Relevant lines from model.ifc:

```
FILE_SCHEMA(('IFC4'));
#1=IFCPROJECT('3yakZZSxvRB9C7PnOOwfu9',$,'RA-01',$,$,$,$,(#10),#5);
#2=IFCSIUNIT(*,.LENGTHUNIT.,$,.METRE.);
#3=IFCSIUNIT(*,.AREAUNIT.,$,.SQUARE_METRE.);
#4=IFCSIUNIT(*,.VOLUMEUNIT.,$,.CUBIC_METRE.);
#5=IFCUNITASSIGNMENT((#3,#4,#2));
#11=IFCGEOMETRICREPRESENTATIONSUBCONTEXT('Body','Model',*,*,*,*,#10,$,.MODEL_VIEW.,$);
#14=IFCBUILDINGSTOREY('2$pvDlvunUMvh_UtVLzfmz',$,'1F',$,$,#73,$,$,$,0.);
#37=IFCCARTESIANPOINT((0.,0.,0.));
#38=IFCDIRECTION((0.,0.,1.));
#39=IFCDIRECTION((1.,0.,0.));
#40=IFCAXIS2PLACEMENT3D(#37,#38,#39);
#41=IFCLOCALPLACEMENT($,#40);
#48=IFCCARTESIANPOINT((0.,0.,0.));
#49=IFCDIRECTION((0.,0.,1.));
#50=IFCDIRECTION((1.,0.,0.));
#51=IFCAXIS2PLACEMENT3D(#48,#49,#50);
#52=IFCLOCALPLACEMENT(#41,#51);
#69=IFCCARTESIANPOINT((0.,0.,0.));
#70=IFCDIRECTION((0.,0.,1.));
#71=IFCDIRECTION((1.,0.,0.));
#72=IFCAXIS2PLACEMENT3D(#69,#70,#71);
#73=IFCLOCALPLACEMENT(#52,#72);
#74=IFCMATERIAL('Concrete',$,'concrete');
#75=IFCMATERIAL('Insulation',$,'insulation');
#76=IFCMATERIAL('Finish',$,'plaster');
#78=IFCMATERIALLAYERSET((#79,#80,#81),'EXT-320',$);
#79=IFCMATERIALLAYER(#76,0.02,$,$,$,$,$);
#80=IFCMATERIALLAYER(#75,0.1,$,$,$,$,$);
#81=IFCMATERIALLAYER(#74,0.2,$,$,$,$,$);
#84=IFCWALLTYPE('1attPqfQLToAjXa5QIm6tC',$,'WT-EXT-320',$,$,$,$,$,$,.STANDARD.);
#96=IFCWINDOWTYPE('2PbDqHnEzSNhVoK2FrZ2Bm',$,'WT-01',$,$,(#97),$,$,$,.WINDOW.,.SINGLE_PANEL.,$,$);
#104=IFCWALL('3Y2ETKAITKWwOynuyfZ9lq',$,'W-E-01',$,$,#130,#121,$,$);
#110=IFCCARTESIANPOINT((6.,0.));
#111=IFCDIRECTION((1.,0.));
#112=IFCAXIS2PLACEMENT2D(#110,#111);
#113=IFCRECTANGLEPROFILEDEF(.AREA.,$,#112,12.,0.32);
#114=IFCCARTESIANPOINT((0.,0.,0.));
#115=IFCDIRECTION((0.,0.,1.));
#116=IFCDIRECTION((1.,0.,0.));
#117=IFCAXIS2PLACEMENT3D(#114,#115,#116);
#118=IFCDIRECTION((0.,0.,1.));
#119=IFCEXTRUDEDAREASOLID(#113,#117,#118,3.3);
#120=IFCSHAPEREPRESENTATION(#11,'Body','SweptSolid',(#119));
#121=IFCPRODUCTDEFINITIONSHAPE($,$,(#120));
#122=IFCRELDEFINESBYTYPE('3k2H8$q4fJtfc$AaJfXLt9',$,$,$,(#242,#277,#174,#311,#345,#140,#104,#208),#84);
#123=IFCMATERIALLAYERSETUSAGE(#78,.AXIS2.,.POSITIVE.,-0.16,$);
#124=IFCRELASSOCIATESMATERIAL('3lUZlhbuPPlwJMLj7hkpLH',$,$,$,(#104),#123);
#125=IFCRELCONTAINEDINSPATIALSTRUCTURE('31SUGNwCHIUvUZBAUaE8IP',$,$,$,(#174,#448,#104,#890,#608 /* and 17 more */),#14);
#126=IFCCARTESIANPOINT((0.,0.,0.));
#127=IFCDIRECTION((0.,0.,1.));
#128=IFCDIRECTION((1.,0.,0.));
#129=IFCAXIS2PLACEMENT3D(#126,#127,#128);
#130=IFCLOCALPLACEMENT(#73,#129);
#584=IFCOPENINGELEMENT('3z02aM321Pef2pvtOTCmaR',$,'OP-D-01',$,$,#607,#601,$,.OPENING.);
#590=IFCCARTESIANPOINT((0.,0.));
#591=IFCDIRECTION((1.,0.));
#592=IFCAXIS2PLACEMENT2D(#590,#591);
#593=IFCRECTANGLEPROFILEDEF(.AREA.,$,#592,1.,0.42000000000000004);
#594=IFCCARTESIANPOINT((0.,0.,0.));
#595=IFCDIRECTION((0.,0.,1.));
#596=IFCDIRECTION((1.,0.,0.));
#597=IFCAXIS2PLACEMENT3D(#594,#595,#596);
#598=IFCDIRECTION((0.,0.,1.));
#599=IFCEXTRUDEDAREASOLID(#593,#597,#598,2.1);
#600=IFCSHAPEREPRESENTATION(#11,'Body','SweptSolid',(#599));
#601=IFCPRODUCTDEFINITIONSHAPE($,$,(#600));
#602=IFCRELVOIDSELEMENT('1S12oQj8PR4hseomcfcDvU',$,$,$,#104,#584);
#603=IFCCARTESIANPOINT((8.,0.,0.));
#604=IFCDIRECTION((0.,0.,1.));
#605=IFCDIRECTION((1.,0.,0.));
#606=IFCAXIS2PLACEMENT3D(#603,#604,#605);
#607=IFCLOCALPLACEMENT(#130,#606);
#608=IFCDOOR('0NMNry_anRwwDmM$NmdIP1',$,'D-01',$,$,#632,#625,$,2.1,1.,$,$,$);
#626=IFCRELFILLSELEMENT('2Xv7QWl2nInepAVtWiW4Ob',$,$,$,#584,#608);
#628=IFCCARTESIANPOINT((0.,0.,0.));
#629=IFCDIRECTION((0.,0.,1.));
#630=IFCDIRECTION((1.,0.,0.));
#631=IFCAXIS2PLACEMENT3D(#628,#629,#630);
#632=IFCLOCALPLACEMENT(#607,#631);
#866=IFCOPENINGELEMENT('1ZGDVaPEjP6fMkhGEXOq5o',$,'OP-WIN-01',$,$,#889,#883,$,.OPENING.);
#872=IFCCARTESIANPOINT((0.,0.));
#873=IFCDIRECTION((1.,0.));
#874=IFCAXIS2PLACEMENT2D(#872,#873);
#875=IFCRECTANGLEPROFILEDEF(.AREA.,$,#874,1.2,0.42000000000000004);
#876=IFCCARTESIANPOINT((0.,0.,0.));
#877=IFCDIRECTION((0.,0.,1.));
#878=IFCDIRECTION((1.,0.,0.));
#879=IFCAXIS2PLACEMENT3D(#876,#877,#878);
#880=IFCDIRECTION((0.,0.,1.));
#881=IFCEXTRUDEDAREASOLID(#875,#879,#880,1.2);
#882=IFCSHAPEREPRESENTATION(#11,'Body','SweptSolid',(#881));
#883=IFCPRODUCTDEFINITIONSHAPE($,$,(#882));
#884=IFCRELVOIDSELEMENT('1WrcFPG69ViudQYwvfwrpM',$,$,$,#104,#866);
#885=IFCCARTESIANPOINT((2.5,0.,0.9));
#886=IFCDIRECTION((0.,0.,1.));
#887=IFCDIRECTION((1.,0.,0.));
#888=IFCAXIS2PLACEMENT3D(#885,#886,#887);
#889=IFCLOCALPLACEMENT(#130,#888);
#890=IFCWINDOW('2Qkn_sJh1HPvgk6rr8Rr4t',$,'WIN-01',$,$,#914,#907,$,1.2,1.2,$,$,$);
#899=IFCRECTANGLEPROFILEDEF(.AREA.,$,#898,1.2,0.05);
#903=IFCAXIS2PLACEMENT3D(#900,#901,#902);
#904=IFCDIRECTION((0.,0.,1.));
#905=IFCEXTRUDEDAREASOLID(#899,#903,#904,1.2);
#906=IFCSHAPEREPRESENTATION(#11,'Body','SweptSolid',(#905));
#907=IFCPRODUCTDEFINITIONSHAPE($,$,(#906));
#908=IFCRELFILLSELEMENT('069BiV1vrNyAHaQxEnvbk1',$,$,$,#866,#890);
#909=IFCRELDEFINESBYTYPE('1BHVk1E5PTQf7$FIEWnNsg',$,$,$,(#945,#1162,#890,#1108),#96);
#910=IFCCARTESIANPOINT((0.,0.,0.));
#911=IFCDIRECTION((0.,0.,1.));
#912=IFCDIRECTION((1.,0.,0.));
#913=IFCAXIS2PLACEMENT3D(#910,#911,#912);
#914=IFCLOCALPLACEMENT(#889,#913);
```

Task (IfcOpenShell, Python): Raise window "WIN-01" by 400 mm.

```python
import numpy as np
import ifcopenshell
import ifcopenshell.api.geometry
import ifcopenshell.util.placement
import ifcopenshell.util.unit

model = ifcopenshell.open("model.ifc")
unit_scale = ifcopenshell.util.unit.calculate_unit_scale(model)

window = model.by_id(890)
opening = window.FillsVoids[0].RelatingOpeningElement
dz = 0.4 / unit_scale

shift = np.array([0.0, 0.0, dz])
# The window is placed relative to its opening, so it follows when the opening moves.
matrix = ifcopenshell.util.placement.get_local_placement(opening.ObjectPlacement)
matrix[:3, 3] += shift
ifcopenshell.api.geometry.edit_object_placement(
    model, product=opening, matrix=matrix, is_si=False, should_transform_children=True
)

print(f"moved by {dz * unit_scale:+.3f} m")

model.write("model-out.ifc")
```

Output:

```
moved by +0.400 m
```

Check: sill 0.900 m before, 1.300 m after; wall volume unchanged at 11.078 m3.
